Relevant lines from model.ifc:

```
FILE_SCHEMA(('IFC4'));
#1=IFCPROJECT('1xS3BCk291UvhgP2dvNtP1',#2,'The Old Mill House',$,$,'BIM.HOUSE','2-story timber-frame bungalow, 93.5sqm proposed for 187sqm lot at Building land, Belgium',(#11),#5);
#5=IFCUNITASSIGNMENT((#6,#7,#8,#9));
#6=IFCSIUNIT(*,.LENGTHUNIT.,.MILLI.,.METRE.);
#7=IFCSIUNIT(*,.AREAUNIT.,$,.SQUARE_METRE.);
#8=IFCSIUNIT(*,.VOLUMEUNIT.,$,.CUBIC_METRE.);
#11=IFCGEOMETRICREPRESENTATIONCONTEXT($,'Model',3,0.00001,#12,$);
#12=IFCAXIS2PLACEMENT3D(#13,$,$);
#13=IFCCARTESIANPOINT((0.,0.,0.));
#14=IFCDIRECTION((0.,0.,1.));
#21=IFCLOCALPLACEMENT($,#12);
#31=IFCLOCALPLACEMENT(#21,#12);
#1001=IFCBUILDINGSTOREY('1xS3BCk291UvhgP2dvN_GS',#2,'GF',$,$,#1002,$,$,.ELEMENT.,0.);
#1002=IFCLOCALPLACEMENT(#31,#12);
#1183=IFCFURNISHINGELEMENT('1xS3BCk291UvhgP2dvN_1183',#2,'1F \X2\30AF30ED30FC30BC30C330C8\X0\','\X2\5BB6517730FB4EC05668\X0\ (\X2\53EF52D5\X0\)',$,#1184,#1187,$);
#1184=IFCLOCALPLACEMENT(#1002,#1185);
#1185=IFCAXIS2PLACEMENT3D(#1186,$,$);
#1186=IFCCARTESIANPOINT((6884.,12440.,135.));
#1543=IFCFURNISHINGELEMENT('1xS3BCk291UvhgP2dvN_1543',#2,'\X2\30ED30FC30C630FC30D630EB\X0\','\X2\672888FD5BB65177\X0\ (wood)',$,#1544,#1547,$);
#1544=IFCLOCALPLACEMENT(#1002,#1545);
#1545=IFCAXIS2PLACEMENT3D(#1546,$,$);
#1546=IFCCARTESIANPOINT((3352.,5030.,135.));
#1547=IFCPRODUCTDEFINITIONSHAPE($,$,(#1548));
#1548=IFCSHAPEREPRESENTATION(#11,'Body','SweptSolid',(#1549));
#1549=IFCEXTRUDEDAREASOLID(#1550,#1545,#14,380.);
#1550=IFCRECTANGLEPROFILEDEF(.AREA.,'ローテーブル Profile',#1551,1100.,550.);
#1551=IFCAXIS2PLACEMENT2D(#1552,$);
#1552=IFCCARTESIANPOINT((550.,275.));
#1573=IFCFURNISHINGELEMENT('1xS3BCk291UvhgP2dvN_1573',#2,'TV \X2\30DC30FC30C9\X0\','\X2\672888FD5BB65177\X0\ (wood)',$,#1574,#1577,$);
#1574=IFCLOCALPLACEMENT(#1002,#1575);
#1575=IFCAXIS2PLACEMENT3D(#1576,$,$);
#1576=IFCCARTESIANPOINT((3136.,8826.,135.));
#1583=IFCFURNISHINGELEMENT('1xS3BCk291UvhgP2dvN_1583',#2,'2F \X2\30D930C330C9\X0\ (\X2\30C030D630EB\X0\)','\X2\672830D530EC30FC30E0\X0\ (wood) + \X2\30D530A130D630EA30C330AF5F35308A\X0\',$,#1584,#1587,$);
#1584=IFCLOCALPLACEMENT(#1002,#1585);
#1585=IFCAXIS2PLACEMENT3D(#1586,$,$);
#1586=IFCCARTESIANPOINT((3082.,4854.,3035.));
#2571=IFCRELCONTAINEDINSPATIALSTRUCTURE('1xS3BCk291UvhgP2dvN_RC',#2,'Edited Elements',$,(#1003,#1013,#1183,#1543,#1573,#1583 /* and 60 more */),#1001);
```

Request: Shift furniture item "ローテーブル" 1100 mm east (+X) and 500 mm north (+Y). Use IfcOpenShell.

```python
import ifcopenshell
import ifcopenshell.api.geometry
import ifcopenshell.util.placement

model = ifcopenshell.open("model.ifc")

item = model.by_id(1543)
matrix = ifcopenshell.util.placement.get_local_placement(item.ObjectPlacement)
matrix[0, 3] += 1100.0
matrix[1, 3] += 500.0
ifcopenshell.api.geometry.edit_object_placement(model, product=item, matrix=matrix, is_si=False)

print(ifcopenshell.util.placement.get_local_placement(item.ObjectPlacement).round(3) + 0.0)

model.write("model-out.ifc")
```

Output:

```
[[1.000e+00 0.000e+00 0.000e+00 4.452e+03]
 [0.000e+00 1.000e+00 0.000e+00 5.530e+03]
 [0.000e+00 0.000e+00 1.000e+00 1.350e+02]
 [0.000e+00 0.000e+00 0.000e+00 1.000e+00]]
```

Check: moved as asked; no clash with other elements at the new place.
